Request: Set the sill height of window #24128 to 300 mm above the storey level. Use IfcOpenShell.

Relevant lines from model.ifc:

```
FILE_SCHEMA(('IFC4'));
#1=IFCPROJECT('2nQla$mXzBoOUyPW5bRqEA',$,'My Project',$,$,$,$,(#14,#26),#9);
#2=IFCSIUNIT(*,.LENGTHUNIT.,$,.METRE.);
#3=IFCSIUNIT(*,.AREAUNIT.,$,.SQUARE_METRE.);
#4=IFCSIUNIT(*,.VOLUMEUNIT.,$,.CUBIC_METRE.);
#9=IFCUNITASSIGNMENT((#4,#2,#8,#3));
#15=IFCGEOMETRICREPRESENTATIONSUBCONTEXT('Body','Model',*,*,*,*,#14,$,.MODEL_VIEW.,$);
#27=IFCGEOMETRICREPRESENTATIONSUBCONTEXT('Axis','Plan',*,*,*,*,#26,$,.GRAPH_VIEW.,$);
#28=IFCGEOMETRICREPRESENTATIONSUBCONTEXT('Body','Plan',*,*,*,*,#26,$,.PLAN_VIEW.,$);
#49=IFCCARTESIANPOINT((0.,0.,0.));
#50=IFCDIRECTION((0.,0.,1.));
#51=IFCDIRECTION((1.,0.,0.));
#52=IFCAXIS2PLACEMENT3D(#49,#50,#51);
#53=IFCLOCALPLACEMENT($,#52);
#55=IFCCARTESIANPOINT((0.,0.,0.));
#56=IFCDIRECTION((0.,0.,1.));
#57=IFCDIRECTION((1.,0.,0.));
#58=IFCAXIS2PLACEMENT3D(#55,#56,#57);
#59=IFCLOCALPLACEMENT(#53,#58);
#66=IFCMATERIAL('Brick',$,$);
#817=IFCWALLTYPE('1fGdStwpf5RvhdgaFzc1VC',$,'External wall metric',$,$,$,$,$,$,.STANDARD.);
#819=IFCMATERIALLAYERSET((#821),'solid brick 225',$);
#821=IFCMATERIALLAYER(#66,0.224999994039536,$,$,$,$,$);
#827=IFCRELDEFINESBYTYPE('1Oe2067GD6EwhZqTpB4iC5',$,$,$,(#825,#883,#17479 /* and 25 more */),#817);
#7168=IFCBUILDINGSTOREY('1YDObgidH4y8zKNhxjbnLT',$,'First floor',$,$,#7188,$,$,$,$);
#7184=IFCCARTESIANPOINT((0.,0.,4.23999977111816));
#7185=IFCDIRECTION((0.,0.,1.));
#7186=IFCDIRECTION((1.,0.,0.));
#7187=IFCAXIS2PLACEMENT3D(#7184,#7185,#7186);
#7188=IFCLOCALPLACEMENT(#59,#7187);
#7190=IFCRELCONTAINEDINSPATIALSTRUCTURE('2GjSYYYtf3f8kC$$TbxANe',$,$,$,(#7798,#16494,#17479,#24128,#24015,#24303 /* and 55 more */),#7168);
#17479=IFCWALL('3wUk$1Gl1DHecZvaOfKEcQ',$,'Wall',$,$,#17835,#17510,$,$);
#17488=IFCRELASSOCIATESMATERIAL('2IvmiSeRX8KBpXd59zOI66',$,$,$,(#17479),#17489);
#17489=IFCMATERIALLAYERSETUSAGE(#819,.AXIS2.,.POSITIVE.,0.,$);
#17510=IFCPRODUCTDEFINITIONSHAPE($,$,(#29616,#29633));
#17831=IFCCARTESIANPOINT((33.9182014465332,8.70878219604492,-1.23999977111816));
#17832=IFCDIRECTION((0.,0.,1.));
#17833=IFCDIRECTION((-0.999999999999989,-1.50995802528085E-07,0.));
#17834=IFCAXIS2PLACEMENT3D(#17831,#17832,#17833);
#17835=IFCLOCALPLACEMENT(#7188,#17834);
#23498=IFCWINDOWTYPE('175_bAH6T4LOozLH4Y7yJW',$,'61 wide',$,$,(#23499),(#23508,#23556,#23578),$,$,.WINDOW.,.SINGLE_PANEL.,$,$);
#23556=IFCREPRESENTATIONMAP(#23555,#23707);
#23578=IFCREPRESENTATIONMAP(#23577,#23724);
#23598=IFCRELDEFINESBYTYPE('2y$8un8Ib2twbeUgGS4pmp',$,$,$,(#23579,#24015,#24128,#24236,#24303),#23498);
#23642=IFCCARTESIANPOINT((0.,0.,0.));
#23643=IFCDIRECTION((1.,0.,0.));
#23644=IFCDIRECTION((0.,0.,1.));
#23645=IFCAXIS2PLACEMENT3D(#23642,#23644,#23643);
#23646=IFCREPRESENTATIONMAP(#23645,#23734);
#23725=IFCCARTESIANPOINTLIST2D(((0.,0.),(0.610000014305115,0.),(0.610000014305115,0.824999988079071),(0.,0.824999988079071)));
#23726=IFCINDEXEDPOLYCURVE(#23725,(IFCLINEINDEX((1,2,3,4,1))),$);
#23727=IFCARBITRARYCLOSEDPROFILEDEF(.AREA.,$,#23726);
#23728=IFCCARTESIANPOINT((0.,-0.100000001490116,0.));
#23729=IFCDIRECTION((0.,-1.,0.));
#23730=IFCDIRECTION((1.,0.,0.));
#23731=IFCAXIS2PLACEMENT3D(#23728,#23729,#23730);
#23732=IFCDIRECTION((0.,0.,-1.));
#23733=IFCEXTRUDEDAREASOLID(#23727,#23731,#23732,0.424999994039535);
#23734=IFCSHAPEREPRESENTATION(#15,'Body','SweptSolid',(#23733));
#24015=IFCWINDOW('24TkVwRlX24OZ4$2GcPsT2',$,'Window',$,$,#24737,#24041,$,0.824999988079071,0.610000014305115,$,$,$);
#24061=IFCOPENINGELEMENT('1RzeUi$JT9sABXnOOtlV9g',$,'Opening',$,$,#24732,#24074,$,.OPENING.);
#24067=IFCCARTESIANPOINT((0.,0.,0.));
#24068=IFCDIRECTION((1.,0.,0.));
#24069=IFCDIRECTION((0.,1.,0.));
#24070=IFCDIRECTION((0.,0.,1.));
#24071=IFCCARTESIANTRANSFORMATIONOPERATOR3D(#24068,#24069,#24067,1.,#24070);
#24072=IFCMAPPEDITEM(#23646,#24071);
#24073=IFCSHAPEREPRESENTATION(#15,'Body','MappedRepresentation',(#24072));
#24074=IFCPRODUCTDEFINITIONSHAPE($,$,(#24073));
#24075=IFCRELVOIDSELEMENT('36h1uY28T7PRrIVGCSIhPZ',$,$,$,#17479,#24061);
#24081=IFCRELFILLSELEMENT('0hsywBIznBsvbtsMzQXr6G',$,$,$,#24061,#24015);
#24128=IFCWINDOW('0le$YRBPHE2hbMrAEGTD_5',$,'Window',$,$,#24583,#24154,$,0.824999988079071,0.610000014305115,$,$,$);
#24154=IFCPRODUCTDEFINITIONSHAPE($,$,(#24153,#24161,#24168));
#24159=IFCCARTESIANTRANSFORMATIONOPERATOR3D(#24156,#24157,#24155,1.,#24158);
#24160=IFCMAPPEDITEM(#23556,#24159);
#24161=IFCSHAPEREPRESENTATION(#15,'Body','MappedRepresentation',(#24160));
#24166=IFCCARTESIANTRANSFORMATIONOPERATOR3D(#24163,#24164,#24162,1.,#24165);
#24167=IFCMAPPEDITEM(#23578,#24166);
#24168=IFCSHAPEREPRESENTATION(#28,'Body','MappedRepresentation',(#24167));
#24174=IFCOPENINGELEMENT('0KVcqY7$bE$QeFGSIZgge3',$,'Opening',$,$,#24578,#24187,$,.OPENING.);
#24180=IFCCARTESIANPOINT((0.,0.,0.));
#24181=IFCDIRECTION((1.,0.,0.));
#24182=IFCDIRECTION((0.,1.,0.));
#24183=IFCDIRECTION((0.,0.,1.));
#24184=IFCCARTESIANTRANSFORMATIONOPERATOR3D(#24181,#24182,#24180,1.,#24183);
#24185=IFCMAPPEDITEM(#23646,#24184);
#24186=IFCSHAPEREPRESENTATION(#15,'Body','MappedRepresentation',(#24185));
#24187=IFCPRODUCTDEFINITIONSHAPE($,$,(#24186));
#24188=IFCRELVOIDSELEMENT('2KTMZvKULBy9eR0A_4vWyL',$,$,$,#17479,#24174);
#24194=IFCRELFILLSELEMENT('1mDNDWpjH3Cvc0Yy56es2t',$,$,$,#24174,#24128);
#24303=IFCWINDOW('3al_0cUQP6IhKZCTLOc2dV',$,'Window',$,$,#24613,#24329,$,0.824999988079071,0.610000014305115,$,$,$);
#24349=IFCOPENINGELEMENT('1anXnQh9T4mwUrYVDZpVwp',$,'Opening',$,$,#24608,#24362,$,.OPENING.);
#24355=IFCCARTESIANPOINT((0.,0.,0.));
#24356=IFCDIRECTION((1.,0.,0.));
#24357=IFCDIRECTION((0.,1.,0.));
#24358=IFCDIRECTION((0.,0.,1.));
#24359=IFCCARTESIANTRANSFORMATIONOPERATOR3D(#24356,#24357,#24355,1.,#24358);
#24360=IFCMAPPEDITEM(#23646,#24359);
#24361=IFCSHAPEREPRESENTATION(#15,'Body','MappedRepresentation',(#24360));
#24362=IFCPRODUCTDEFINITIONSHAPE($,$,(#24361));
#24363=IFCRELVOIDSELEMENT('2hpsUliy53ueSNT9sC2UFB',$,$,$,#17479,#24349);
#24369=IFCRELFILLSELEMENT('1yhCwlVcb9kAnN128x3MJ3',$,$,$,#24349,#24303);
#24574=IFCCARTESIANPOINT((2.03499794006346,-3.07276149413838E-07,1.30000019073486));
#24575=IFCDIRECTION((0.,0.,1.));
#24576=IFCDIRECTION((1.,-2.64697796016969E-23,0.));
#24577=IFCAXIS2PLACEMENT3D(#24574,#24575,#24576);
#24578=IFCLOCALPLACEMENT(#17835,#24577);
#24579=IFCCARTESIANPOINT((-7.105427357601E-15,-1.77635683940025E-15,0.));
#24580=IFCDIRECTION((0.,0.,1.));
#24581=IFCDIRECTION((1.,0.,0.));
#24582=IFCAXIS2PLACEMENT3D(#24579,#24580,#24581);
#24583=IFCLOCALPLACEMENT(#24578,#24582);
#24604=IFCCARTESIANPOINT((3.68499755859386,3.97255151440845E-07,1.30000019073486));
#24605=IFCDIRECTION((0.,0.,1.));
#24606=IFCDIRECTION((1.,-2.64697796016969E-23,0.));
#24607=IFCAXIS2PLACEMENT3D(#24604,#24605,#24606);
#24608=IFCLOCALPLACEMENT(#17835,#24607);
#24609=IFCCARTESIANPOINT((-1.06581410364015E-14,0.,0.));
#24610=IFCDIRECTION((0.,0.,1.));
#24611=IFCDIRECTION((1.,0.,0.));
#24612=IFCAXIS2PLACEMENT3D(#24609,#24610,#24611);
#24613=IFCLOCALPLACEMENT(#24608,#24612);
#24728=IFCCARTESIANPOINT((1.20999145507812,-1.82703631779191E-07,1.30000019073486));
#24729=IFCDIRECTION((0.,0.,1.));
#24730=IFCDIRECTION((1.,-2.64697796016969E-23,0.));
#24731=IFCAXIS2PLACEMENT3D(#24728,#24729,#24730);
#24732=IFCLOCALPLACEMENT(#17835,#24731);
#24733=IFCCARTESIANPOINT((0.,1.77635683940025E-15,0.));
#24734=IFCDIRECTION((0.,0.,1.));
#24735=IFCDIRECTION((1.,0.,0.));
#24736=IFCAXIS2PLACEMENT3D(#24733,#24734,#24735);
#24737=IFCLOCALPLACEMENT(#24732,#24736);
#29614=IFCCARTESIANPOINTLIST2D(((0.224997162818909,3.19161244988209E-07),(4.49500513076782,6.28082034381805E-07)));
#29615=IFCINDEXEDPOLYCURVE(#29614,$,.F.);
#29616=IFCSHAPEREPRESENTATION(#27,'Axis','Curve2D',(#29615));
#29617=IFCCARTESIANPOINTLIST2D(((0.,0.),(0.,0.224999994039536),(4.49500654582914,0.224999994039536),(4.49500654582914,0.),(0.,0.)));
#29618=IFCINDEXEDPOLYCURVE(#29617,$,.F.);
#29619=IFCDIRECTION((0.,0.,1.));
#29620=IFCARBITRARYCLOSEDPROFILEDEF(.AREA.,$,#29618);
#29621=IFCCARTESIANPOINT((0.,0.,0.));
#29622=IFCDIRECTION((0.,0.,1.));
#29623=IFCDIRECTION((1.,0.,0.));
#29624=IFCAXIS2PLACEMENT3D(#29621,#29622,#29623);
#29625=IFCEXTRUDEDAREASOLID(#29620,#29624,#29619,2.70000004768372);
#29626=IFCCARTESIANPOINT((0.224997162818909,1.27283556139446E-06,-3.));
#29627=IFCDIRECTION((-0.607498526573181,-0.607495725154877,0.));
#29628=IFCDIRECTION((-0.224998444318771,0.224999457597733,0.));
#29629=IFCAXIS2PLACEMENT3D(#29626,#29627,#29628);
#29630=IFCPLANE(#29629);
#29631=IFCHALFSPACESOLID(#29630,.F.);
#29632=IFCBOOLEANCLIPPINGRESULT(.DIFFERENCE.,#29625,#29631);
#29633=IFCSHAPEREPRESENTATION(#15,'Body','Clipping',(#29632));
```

```python
import numpy as np
import ifcopenshell
import ifcopenshell.api.geometry
import ifcopenshell.geom
import ifcopenshell.util.element
import ifcopenshell.util.placement
import ifcopenshell.util.shape
import ifcopenshell.util.unit

model = ifcopenshell.open("model.ifc")
unit_scale = ifcopenshell.util.unit.calculate_unit_scale(model)

window = model.by_guid("0le$YRBPHE2hbMrAEGTD_5")
opening = window.FillsVoids[0].RelatingOpeningElement
storey = ifcopenshell.util.element.get_container(window, ifc_class="IfcBuildingStorey")
level = ifcopenshell.util.placement.get_local_placement(storey.ObjectPlacement)[2, 3]

# The opening's origin need not be at the sill, so measure its lowest point.
shape = ifcopenshell.geom.create_shape(ifcopenshell.geom.settings(), opening)
bottom = ifcopenshell.util.shape.get_shape_bottom_elevation(shape, shape.geometry) / unit_scale
dz = level + 0.3 / unit_scale - bottom

shift = np.array([0.0, 0.0, dz])
# The window is placed relative to its opening, so it follows when the opening moves.
matrix = ifcopenshell.util.placement.get_local_placement(opening.ObjectPlacement)
matrix[:3, 3] += shift
ifcopenshell.api.geometry.edit_object_placement(
    model, product=opening, matrix=matrix, is_si=False, should_transform_children=True
)

print(f"moved by {dz * unit_scale:+.3f} m")

model.write("model_v2.ifc")
```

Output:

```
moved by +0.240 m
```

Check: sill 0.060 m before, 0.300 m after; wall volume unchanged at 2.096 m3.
